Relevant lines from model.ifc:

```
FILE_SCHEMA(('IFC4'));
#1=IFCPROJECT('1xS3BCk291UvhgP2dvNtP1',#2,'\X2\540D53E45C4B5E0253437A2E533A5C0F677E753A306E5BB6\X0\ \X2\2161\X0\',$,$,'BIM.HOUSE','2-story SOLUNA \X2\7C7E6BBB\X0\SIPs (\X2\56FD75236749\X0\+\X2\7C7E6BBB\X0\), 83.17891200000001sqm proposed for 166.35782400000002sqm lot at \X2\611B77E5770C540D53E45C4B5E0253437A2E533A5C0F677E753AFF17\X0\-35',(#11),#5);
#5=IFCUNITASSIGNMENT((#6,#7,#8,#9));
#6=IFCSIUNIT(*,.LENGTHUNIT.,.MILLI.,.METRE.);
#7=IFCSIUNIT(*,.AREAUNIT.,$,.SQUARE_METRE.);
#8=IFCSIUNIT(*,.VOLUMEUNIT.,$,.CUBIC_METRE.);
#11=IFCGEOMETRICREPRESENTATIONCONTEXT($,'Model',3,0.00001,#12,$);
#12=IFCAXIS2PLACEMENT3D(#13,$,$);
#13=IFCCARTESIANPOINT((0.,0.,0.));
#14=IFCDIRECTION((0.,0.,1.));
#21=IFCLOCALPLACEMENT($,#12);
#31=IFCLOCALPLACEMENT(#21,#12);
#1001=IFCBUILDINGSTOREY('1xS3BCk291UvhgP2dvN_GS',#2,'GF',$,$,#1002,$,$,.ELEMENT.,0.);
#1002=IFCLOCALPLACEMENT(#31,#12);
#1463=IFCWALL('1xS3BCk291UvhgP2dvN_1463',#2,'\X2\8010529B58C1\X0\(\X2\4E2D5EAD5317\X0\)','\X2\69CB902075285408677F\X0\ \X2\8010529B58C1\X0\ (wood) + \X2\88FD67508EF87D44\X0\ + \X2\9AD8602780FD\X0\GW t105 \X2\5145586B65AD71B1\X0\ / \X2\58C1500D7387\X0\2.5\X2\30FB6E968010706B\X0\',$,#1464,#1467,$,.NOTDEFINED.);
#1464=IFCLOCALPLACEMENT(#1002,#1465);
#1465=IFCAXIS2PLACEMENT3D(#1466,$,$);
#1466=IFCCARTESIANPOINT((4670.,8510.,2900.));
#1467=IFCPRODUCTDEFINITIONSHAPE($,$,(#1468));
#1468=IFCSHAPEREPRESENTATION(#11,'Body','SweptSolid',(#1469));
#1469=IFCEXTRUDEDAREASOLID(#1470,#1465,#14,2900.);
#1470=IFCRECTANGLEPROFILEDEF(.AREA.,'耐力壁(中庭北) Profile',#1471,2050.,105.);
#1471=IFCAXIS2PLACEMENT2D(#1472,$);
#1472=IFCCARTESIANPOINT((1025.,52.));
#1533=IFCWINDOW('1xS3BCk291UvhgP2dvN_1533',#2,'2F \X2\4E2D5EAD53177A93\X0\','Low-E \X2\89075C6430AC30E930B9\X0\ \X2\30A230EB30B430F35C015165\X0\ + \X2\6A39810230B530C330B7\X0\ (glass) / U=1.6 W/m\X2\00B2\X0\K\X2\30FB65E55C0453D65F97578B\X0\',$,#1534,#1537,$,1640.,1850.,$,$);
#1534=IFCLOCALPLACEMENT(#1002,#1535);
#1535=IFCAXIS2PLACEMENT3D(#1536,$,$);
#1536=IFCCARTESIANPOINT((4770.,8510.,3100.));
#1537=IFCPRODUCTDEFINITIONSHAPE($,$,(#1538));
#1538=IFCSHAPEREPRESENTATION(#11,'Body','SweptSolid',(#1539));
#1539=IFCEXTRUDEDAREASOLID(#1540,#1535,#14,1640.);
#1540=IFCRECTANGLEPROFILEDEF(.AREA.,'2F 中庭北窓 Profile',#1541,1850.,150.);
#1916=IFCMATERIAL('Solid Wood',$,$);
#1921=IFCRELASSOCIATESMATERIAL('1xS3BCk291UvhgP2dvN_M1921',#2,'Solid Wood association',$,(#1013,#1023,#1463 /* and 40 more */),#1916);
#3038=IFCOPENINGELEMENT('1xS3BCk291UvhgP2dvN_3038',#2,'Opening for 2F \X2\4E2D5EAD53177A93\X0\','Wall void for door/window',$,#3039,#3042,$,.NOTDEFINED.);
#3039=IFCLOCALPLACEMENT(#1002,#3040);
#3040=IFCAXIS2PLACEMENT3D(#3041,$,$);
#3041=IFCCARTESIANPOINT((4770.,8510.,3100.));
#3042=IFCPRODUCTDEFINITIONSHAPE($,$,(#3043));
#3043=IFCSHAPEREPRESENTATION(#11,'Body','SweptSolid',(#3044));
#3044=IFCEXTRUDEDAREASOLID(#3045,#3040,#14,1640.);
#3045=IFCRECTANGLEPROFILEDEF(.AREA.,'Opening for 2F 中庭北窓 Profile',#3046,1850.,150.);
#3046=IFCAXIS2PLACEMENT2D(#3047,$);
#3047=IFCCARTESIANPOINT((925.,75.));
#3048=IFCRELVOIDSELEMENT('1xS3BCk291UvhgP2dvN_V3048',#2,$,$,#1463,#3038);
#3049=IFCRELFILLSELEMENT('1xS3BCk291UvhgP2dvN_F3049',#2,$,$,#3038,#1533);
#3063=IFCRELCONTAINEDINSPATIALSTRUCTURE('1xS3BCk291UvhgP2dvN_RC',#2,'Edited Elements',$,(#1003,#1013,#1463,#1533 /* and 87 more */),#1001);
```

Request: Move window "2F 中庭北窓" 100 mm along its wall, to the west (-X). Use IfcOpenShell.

```python
import ifcopenshell
import ifcopenshell.api.geometry
import ifcopenshell.util.placement

model = ifcopenshell.open("model.ifc")

window = model.by_id(1533)
opening = window.FillsVoids[0].RelatingOpeningElement
wall = opening.VoidsElements[0].RelatingBuildingElement

wall_matrix = ifcopenshell.util.placement.get_local_placement(wall.ObjectPlacement)
shift = wall_matrix[:3, 0] * -100.0
before = ifcopenshell.util.placement.get_local_placement(window.ObjectPlacement)[:3, 3].copy()

# The window is not placed relative to its opening, so move both.
for product in (opening, window):
    matrix = ifcopenshell.util.placement.get_local_placement(product.ObjectPlacement)
    matrix[:3, 3] += shift
    ifcopenshell.api.geometry.edit_object_placement(model, product=product, matrix=matrix, is_si=False)

after = ifcopenshell.util.placement.get_local_placement(window.ObjectPlacement)[:3, 3]
print("window moved by", (after - before).round(3) + 0.0)

model.write("model_rev.ifc")
```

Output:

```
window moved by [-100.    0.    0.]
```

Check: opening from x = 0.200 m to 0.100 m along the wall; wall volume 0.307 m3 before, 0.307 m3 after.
